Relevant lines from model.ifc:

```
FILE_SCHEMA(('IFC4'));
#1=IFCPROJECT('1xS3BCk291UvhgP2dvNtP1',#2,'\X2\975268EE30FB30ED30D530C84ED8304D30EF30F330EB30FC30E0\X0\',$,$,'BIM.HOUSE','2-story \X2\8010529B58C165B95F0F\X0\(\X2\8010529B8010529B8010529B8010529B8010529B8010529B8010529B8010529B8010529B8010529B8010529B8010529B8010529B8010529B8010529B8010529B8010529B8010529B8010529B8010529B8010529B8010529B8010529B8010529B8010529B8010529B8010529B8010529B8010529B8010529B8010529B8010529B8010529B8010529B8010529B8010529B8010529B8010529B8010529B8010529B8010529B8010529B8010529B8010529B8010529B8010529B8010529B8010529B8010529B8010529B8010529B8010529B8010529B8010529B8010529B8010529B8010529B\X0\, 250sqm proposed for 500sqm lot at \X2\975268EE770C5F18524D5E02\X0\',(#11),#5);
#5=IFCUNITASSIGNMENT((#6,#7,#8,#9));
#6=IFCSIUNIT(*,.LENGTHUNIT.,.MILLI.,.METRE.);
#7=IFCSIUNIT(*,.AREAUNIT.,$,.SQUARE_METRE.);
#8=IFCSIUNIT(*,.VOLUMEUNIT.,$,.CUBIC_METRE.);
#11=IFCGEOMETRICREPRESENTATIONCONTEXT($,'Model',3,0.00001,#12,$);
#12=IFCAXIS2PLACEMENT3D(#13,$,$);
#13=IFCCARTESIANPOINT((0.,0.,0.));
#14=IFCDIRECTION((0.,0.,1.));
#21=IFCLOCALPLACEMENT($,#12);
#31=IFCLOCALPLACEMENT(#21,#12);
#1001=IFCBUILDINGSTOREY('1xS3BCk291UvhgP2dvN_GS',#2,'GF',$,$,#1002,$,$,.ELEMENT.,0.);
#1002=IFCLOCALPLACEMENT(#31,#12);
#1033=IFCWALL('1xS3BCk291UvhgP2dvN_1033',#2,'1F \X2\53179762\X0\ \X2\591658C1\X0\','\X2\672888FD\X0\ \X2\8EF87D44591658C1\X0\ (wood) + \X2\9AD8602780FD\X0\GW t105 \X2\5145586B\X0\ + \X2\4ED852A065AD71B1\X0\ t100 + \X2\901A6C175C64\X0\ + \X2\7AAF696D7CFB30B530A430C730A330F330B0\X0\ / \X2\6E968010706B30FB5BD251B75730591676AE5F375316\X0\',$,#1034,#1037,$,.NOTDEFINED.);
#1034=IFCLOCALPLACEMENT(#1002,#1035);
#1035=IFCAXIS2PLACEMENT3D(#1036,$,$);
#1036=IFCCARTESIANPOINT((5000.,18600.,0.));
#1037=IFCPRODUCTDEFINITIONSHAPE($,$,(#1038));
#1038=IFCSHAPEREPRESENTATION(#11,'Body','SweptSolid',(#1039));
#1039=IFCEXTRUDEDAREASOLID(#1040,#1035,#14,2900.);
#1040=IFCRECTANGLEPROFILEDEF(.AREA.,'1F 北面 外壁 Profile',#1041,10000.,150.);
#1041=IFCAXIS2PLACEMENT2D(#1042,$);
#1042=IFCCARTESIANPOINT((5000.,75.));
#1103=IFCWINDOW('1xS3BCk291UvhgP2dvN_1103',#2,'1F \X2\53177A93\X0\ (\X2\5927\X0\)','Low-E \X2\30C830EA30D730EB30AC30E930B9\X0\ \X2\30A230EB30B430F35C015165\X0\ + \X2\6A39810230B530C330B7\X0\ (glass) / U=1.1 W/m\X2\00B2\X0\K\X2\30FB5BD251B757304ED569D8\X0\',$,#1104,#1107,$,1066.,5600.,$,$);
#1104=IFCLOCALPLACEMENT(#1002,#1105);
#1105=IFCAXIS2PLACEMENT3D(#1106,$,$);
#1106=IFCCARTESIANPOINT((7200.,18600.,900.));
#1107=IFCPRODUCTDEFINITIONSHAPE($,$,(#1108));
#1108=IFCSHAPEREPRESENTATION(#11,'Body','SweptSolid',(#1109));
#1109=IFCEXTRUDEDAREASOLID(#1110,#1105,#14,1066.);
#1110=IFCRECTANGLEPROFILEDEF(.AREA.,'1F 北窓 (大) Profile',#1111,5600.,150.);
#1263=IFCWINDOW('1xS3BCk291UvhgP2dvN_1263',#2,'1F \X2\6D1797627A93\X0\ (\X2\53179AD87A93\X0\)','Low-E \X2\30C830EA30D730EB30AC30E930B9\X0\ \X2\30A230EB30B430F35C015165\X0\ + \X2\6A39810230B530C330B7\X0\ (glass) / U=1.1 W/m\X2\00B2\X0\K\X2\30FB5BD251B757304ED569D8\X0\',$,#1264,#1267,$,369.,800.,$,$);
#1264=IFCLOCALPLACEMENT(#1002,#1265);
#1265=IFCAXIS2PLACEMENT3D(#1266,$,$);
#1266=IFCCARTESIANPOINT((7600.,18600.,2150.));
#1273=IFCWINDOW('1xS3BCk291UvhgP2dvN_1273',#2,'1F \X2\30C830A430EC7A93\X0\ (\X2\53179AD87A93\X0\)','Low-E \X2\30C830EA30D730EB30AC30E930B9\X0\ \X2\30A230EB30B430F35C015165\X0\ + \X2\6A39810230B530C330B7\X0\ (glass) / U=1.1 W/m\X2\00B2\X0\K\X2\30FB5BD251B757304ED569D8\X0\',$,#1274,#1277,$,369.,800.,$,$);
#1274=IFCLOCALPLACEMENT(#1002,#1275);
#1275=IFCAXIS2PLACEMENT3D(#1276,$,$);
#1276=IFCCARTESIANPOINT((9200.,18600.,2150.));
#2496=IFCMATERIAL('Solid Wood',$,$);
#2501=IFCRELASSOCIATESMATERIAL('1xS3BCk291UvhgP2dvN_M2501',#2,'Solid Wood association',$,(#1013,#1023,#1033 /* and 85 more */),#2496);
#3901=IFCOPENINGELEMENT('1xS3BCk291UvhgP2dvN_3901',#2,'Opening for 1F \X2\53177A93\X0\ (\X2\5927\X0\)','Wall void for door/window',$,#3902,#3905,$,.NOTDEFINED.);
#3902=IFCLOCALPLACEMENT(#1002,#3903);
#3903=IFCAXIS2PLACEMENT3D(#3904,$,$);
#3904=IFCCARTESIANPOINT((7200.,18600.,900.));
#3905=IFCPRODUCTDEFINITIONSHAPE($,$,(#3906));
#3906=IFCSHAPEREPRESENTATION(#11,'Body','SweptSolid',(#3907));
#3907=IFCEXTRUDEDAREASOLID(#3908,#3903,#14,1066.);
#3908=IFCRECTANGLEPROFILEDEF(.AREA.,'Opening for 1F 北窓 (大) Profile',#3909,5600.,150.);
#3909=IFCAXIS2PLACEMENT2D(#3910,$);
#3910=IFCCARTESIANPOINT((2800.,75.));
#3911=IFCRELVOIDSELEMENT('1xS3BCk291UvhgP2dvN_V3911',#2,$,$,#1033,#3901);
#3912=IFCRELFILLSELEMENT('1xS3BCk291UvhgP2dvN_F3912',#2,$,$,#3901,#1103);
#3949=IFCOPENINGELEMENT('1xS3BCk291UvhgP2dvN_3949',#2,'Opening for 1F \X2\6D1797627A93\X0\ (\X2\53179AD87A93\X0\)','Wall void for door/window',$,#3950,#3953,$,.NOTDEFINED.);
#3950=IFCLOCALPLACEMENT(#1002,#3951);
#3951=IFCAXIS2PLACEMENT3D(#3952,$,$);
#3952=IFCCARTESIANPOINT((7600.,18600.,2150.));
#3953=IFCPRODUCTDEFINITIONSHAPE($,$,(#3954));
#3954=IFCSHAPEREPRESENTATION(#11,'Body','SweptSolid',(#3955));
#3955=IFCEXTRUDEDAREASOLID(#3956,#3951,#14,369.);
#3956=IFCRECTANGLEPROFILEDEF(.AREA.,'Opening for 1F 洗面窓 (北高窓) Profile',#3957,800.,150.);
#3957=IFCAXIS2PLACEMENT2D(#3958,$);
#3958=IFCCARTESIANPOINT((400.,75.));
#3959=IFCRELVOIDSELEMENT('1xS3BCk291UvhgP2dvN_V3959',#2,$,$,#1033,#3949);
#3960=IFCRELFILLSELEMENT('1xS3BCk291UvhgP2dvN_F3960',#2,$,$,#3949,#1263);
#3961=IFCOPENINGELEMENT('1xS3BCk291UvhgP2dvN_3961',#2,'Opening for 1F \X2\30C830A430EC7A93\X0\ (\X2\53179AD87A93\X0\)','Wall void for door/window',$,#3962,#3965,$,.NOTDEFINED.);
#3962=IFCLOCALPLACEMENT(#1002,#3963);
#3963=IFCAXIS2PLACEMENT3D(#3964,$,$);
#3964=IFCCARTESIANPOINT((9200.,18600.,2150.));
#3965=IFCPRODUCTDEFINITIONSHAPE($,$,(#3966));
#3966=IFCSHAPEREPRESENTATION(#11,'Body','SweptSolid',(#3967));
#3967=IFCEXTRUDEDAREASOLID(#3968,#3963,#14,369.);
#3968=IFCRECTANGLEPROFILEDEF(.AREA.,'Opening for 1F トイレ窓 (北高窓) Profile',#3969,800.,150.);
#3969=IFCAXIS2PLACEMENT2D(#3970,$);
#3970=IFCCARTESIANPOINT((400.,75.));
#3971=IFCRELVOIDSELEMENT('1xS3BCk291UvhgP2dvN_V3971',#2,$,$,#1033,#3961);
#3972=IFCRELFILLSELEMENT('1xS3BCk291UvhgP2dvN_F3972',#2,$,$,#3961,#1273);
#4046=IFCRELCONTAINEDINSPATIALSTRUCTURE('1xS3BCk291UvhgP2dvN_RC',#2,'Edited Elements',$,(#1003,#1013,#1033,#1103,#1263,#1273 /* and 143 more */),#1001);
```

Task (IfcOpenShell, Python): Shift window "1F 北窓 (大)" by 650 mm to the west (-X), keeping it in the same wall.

```python
import ifcopenshell
import ifcopenshell.api.geometry
import ifcopenshell.util.placement

model = ifcopenshell.open("model.ifc")

window = model.by_guid("1xS3BCk291UvhgP2dvN_1103")
opening = window.FillsVoids[0].RelatingOpeningElement
wall = opening.VoidsElements[0].RelatingBuildingElement

wall_matrix = ifcopenshell.util.placement.get_local_placement(wall.ObjectPlacement)
shift = wall_matrix[:3, 0] * -650.0
before = ifcopenshell.util.placement.get_local_placement(window.ObjectPlacement)[:3, 3].copy()

# The window is not placed relative to its opening, so move both.
for product in (opening, window):
    matrix = ifcopenshell.util.placement.get_local_placement(product.ObjectPlacement)
    matrix[:3, 3] += shift
    ifcopenshell.api.geometry.edit_object_placement(model, product=product, matrix=matrix, is_si=False)

after = ifcopenshell.util.placement.get_local_placement(window.ObjectPlacement)[:3, 3]
print("window moved by", (after - before).round(3) + 0.0)

model.write("model-out.ifc")
```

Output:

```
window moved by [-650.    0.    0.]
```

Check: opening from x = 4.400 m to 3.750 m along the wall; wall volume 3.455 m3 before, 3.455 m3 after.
